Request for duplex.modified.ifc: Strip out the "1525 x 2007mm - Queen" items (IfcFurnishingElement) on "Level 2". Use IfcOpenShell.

First a look at what the model holds.

```python
import ifcopenshell
import ifcopenshell.util.element

model = ifcopenshell.open("duplex.modified.ifc")
print(model.schema)
storey = next(s for s in model.by_type("IfcBuildingStorey") if s.Name == "Level 2")
furniture = [e for e in ifcopenshell.util.element.get_decomposition(storey) if e.is_a("IfcFurnishingElement")]
seen = {}
for e in furniture:
    element_type = ifcopenshell.util.element.get_type(e)
    name = element_type.Name if element_type not in (None, e) else None
    seen[name] = seen.get(name, 0) + 1
for name, count in sorted(seen.items(), key=str):
    print(count, "x", name)
```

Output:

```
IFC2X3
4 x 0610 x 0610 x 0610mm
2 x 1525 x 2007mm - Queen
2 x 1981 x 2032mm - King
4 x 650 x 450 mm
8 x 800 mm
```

```python
import ifcopenshell
import ifcopenshell.api.root
import ifcopenshell.util.element

model = ifcopenshell.open("duplex.modified.ifc")

storey = next(s for s in model.by_type("IfcBuildingStorey") if s.Name == "Level 2")
furniture = [e for e in ifcopenshell.util.element.get_decomposition(storey) if e.is_a("IfcFurnishingElement")]
targets = [e for e in furniture if (t := ifcopenshell.util.element.get_type(e)) not in (None, e) and t.Name == "1525 x 2007mm - Queen"]

for e in targets:
    ifcopenshell.api.root.remove_product(model, product=e)
print(len(targets), "removed")

model.write("duplex.modified_edited.ifc")
```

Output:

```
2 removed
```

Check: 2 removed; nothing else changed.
